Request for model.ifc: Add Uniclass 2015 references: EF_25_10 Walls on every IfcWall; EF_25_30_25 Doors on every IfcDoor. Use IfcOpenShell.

First a look at what the model holds.

```python
import ifcopenshell

model = ifcopenshell.open("model.ifc")
print(model.schema)
print("classifications:", [c.Name for c in model.by_type("IfcClassification")])
for ifc_class in ("IfcDoor", "IfcRoof", "IfcStair", "IfcWall", "IfcWindow"):
    print(ifc_class, len(model.by_type(ifc_class)))
```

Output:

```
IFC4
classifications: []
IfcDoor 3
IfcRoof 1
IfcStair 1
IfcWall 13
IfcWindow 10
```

```python
import ifcopenshell
import ifcopenshell.api.classification

model = ifcopenshell.open("model.ifc")

system = ifcopenshell.api.classification.add_classification(model, classification="Uniclass 2015")

codes = {
    "IfcWall": ("EF_25_10", "Walls"),
    "IfcDoor": ("EF_25_30_25", "Doors"),
}
for ifc_class, (code, name) in codes.items():
    products = model.by_type(ifc_class)
    ifcopenshell.api.classification.add_reference(
        model, products=products, classification=system, identification=code, name=name
    )
    print(code, len(products))

model.write("model_rev.ifc")
```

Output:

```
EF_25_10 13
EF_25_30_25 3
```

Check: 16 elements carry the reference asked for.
